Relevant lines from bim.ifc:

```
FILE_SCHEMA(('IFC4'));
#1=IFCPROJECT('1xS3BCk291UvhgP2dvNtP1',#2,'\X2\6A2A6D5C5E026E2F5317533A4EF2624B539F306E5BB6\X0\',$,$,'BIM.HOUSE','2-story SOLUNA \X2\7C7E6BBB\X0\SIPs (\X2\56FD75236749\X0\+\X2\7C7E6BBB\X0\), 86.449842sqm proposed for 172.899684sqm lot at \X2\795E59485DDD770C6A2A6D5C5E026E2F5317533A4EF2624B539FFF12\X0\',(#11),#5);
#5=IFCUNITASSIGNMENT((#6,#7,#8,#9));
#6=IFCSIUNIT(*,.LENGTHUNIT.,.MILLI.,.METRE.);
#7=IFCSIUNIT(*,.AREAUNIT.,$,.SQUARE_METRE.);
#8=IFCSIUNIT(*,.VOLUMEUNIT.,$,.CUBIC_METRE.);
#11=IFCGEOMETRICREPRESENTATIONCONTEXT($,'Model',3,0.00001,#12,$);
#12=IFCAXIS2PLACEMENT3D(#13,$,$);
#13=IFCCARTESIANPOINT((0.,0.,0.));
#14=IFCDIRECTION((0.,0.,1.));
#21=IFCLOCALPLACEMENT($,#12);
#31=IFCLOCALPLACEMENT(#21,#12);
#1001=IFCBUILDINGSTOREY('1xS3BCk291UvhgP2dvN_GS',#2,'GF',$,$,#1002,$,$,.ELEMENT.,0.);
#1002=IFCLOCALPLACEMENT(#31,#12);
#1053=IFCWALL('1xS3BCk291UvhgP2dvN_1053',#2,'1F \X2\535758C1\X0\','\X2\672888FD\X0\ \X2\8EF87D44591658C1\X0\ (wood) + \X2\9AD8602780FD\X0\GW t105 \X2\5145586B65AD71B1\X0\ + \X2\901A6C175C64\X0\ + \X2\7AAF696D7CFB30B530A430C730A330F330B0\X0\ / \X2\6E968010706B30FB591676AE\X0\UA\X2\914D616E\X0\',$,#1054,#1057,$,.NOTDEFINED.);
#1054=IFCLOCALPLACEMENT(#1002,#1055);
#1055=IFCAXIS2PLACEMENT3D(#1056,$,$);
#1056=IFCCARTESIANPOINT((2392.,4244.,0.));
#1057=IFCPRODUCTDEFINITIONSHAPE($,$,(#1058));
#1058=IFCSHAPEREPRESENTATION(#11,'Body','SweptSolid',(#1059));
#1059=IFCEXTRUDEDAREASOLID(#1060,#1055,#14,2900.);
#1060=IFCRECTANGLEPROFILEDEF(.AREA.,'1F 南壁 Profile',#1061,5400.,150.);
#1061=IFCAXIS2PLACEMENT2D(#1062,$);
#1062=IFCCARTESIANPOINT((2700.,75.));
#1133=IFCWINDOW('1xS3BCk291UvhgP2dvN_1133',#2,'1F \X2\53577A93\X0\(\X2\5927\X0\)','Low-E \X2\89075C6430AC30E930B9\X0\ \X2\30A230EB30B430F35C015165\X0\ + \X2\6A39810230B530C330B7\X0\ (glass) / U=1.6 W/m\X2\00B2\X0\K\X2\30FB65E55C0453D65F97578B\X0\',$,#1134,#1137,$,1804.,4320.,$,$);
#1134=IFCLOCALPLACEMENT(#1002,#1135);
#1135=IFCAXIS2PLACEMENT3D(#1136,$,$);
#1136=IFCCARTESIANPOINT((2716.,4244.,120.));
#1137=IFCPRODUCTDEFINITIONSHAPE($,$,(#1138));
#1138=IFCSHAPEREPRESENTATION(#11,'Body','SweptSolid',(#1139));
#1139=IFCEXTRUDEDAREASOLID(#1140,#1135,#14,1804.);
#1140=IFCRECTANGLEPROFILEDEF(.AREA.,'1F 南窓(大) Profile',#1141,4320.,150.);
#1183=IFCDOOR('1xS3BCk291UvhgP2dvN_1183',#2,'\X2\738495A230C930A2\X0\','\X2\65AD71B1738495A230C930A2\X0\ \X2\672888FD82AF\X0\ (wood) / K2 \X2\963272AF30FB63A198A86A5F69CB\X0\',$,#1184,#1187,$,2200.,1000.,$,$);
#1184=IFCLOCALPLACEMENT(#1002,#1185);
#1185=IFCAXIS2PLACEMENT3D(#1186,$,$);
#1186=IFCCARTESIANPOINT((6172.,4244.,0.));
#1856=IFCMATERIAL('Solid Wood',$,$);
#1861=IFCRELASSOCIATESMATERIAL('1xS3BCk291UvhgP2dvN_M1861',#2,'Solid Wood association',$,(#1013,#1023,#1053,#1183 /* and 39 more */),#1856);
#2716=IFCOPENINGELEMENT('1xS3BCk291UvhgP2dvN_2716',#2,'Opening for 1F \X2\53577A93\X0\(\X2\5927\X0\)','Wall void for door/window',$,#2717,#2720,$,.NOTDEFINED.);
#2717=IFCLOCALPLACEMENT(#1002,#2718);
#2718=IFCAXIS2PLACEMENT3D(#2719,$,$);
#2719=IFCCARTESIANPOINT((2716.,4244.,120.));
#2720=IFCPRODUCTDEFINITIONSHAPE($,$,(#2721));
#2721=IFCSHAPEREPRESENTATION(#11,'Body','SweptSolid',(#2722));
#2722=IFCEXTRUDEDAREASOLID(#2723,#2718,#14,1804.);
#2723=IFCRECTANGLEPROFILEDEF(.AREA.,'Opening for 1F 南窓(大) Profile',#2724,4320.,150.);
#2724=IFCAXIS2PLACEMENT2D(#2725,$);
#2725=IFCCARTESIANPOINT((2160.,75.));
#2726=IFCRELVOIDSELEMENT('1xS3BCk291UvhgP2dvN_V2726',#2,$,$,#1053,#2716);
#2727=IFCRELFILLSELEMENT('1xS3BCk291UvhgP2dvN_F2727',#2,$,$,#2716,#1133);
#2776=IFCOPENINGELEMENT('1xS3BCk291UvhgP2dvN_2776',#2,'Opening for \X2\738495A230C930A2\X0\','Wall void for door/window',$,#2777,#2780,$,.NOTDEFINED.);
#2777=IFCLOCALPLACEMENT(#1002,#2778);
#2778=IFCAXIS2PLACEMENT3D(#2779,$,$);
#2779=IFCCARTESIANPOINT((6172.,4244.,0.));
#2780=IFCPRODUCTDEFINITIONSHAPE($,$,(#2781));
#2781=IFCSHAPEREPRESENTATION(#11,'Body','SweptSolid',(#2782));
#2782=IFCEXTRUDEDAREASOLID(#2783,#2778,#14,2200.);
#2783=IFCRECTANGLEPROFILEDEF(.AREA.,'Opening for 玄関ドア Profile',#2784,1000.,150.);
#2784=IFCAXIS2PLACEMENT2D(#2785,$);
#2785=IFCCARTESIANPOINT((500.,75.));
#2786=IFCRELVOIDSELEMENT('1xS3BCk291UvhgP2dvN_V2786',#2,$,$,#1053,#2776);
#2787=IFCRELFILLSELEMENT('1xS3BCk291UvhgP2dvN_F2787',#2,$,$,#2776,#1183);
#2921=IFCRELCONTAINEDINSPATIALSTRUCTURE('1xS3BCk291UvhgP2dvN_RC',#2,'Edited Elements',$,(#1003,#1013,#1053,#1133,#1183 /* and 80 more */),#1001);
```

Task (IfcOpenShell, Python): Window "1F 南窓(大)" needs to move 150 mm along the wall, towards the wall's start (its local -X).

```python
import ifcopenshell
import ifcopenshell.api.geometry
import ifcopenshell.util.placement
import ifcopenshell.util.unit

model = ifcopenshell.open("bim.ifc")
unit_scale = ifcopenshell.util.unit.calculate_unit_scale(model)

window = model.by_guid("1xS3BCk291UvhgP2dvN_1133")
opening = window.FillsVoids[0].RelatingOpeningElement
wall = opening.VoidsElements[0].RelatingBuildingElement

wall_matrix = ifcopenshell.util.placement.get_local_placement(wall.ObjectPlacement)
shift = wall_matrix[:3, 0] * -0.15 / unit_scale
before = ifcopenshell.util.placement.get_local_placement(window.ObjectPlacement)[:3, 3].copy()

# The window is not placed relative to its opening, so move both.
for product in (opening, window):
    matrix = ifcopenshell.util.placement.get_local_placement(product.ObjectPlacement)
    matrix[:3, 3] += shift
    ifcopenshell.api.geometry.edit_object_placement(model, product=product, matrix=matrix, is_si=False)

after = ifcopenshell.util.placement.get_local_placement(window.ObjectPlacement)[:3, 3]
print("window moved by", (after - before).round(3) + 0.0)

model.write("bim-out.ifc")
```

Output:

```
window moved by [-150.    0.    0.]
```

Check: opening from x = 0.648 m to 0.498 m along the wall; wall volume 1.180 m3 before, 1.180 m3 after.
